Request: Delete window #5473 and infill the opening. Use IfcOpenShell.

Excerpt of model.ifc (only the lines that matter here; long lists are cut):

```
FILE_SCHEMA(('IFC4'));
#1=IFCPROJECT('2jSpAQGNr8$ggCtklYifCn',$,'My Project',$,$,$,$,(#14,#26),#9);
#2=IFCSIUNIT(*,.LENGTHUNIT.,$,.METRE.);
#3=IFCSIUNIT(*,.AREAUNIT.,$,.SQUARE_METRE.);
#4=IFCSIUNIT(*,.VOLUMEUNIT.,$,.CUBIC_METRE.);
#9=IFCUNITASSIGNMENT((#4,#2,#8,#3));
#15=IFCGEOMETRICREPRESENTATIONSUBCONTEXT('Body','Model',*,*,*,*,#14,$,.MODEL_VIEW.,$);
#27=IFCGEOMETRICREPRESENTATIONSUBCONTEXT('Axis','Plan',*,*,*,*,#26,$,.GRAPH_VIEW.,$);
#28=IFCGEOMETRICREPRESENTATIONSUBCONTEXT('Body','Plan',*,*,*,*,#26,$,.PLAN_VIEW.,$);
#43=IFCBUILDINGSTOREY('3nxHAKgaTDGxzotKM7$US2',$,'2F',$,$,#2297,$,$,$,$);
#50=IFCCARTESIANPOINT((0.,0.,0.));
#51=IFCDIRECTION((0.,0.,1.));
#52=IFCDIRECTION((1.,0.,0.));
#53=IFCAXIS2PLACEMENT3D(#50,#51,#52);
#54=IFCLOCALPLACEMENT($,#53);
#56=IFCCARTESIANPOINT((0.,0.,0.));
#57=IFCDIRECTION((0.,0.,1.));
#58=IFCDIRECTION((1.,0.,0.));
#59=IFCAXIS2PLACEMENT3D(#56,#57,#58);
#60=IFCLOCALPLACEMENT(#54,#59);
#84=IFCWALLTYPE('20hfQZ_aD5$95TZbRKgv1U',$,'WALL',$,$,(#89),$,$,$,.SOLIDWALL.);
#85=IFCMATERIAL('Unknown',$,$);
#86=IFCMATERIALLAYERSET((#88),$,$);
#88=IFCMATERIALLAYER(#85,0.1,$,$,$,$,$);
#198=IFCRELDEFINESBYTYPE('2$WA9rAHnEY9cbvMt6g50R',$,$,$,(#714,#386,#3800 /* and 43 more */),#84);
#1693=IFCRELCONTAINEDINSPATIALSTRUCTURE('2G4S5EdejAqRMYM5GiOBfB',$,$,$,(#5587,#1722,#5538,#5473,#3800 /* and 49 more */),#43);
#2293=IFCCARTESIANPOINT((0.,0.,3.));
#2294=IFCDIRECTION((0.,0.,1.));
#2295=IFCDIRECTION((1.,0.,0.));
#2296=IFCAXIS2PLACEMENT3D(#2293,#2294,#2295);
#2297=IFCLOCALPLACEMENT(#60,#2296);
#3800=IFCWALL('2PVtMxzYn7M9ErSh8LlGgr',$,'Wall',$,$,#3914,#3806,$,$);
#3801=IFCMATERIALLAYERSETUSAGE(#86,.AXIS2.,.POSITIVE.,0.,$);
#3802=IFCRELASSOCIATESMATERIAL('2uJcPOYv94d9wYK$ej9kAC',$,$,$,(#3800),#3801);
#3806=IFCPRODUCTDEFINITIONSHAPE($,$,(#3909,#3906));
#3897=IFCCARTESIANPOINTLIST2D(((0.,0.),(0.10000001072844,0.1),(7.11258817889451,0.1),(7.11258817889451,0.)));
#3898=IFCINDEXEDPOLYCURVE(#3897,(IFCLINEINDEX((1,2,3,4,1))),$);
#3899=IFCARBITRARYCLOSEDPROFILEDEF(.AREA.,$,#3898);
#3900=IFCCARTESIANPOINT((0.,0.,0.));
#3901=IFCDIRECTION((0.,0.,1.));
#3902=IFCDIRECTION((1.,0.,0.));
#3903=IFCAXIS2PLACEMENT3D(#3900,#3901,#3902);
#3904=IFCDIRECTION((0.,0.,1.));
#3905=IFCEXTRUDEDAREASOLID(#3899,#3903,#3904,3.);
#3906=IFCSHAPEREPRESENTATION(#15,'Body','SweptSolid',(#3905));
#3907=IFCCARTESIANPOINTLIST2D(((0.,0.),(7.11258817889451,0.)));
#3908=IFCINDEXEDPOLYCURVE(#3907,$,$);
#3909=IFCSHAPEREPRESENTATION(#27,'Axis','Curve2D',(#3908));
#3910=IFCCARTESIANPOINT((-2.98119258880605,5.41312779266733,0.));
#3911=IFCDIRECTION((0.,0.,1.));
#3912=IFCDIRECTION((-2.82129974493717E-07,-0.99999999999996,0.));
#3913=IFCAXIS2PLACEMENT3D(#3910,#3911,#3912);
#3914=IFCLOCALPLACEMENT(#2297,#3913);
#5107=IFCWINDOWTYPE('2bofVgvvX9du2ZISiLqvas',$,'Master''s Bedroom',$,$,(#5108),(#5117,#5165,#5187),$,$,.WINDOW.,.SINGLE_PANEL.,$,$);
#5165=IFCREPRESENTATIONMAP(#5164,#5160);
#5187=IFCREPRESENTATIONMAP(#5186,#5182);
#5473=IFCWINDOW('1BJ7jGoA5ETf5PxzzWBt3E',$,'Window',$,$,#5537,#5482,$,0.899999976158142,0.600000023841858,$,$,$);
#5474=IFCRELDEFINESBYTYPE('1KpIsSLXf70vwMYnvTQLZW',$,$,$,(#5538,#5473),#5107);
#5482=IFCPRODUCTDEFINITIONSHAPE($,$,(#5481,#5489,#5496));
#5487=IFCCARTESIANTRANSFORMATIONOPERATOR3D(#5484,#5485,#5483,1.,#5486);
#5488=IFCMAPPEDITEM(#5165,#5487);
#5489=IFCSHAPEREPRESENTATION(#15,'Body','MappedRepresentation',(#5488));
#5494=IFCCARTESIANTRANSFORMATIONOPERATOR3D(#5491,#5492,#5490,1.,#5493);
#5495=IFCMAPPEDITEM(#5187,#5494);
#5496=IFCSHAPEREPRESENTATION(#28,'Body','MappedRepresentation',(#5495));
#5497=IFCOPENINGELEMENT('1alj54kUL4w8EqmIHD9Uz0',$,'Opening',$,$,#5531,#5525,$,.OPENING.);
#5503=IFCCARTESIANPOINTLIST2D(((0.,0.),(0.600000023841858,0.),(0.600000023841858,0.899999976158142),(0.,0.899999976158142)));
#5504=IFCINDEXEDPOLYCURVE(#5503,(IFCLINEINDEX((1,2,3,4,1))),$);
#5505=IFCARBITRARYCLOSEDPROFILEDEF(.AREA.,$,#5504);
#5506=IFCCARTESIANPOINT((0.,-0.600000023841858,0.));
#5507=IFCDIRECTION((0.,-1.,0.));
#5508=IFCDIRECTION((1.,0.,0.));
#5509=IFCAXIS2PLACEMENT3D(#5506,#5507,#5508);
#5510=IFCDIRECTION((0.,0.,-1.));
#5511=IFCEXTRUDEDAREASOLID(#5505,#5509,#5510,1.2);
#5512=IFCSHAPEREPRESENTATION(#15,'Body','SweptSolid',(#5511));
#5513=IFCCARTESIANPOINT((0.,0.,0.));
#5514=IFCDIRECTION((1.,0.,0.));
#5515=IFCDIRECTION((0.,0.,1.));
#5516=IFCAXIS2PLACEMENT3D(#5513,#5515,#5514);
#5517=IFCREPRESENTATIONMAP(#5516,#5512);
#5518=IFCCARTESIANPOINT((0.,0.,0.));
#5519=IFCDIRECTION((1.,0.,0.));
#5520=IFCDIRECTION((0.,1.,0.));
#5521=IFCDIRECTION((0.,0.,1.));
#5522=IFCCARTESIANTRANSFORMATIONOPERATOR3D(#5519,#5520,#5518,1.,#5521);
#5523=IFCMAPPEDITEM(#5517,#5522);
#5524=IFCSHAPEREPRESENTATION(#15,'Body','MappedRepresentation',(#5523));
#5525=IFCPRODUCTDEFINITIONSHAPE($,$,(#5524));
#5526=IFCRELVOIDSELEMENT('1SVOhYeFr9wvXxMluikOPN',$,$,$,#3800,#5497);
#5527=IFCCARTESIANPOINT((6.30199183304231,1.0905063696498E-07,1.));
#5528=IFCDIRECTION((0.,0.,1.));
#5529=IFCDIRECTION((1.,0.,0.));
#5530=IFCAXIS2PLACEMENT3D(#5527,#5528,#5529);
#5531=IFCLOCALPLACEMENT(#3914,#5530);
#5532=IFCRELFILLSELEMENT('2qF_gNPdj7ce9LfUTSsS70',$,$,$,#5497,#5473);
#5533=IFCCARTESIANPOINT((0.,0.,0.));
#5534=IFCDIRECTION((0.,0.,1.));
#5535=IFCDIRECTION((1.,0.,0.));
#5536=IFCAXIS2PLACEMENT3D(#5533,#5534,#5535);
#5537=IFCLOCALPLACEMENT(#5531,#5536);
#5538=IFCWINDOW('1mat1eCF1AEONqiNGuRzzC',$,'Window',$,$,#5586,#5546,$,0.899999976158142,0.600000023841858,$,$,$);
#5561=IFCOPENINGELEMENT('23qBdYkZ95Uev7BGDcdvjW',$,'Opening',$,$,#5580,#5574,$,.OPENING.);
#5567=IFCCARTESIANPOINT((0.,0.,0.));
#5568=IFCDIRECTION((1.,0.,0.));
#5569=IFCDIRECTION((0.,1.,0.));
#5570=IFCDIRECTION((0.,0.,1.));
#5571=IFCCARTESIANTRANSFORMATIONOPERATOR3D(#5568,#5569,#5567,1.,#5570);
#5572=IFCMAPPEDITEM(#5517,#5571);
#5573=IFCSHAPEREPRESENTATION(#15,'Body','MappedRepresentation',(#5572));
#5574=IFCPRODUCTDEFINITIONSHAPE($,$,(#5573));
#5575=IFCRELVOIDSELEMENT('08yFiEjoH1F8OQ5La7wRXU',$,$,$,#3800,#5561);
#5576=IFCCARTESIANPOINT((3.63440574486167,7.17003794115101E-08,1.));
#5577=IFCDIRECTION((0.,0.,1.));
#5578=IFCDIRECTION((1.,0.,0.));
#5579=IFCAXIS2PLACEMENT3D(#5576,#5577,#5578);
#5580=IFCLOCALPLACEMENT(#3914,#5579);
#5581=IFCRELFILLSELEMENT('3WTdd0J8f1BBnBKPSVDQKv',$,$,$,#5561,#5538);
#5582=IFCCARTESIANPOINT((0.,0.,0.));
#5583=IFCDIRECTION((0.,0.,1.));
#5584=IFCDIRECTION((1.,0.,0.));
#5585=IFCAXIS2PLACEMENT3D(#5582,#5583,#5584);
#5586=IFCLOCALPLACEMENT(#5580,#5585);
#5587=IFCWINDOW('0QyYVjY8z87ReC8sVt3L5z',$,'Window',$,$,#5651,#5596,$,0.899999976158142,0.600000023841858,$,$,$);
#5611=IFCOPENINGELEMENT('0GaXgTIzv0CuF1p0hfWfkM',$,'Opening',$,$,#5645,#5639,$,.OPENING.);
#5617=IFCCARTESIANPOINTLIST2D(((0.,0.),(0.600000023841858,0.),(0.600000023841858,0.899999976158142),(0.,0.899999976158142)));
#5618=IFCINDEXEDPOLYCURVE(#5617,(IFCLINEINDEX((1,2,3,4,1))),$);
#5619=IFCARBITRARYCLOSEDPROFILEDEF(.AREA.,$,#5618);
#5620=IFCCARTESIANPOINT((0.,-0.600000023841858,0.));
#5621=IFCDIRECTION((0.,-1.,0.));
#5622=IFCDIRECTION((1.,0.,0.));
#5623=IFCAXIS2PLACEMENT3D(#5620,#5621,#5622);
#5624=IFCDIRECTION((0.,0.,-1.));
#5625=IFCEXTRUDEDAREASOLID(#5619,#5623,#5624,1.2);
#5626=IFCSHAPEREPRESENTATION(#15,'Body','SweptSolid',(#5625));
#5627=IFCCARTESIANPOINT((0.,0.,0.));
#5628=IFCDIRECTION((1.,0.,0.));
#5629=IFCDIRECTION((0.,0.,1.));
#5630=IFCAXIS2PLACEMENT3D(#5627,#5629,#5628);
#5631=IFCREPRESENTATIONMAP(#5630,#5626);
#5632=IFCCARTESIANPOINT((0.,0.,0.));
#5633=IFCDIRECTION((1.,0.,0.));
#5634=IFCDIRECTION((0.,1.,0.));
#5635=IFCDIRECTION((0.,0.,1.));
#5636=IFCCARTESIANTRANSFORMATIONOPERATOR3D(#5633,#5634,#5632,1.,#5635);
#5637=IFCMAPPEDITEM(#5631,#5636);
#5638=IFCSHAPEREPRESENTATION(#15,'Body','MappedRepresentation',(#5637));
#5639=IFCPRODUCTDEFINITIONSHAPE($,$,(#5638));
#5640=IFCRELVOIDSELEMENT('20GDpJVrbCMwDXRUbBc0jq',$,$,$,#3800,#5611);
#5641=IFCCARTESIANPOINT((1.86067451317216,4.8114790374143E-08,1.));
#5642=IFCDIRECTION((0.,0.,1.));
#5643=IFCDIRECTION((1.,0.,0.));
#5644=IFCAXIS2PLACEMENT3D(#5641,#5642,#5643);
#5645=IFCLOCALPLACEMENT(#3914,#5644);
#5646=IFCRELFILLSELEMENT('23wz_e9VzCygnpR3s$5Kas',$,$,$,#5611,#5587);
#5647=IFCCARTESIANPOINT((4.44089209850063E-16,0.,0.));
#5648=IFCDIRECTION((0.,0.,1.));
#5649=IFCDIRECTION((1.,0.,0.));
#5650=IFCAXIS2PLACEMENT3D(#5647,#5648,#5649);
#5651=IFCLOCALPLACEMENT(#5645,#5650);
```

```python
import ifcopenshell
import ifcopenshell.api.feature
import ifcopenshell.api.root
import ifcopenshell.geom
import ifcopenshell.util.shape

model = ifcopenshell.open("model.ifc")
settings = ifcopenshell.geom.settings()


def volume(element):
    """Net volume in cubic metres, openings subtracted."""
    shape = ifcopenshell.geom.create_shape(settings, element)
    return ifcopenshell.util.shape.get_volume(shape.geometry)


window = model.by_guid("1BJ7jGoA5ETf5PxzzWBt3E")
opening = window.FillsVoids[0].RelatingOpeningElement
wall = opening.VoidsElements[0].RelatingBuildingElement
before = volume(wall)

ifcopenshell.api.root.remove_product(model, product=window)
ifcopenshell.api.feature.remove_feature(model, feature=opening)

after = volume(wall)

print(f"wall volume {before:.3f} -> {after:.3f} m3")

model.write("model_rev.ifc")
```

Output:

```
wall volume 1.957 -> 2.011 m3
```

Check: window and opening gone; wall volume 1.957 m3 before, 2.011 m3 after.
